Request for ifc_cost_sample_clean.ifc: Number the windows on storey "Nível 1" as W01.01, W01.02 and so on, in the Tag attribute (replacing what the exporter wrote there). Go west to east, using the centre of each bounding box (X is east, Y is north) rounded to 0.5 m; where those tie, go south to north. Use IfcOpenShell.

First a look at what the model holds.

```python
import ifcopenshell
import ifcopenshell.util.element
import ifcopenshell.util.placement

model = ifcopenshell.open("ifc_cost_sample_clean.ifc")
print(model.schema)
storey = next(s for s in model.by_type("IfcBuildingStorey") if s.Name == "Nível 1")
windows = [e for e in ifcopenshell.util.element.get_decomposition(storey) if e.is_a("IfcWindow")]
for e in sorted(windows, key=lambda e: e.id()):
    origin = ifcopenshell.util.placement.get_local_placement(e.ObjectPlacement)[:3, 3]
    print(e.id(), e.Tag, e.Name, origin.round(2) + 0.0, sep=" | ")
```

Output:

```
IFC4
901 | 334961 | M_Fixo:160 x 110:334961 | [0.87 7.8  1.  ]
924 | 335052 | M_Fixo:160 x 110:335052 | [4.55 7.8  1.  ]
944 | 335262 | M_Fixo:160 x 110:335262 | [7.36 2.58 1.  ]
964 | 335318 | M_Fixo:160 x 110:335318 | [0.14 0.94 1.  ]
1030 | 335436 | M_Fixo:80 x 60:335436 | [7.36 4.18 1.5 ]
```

```python
import ifcopenshell
import ifcopenshell.geom
import ifcopenshell.util.element
import ifcopenshell.util.shape

model = ifcopenshell.open("ifc_cost_sample_clean.ifc")
settings = ifcopenshell.geom.settings()
settings.set("use-world-coords", True)


def centre(element):
    shape = ifcopenshell.geom.create_shape(settings, element)
    return ifcopenshell.util.shape.get_bbox_centroid(shape.geometry)


storey = next(s for s in model.by_type("IfcBuildingStorey") if s.Name == "Nível 1")
windows = [e for e in ifcopenshell.util.element.get_decomposition(storey) if e.is_a("IfcWindow")]

# Insertion points can sit at a corner or the storey origin, so sort by the geometry (in metres).
centres = {e: centre(e) for e in windows}
windows.sort(key=lambda e: (round(centres[e][0] / 0.5), centres[e][1]))

for i, e in enumerate(windows, start=1):
    number = f"W01.{i:02d}"
    e.Tag = number
    print(e.id(), number)

model.write("ifc_cost_sample_clean_rev.ifc")
```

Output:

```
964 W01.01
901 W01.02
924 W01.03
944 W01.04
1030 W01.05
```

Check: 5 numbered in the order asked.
